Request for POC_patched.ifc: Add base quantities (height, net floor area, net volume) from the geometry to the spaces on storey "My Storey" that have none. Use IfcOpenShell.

First a look at what the model holds.

```python
import ifcopenshell
import ifcopenshell.util.element
import ifcopenshell.util.unit

model = ifcopenshell.open("POC_patched.ifc")
print(model.schema)
for unit_type in ("LENGTHUNIT", "AREAUNIT", "VOLUMEUNIT"):
    print(unit_type, ifcopenshell.util.unit.calculate_unit_scale(model, unit_type))
storey = next(s for s in model.by_type("IfcBuildingStorey") if s.Name == "My Storey")
spaces = [e for e in ifcopenshell.util.element.get_decomposition(storey) if e.is_a("IfcSpace")]
for e in sorted(spaces, key=lambda e: e.id()):
    print(e.id(), e.is_a(), e.Name, list(ifcopenshell.util.element.get_psets(e, qtos_only=True)), sep=" | ")
```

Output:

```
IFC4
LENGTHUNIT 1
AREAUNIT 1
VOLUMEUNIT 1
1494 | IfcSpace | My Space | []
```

```python
import ifcopenshell
import ifcopenshell.api.pset
import ifcopenshell.geom
import ifcopenshell.util.element
import ifcopenshell.util.shape
import ifcopenshell.util.unit

model = ifcopenshell.open("POC_patched.ifc")
unit_scale = ifcopenshell.util.unit.calculate_unit_scale(model)
area_scale = ifcopenshell.util.unit.calculate_unit_scale(model, "AREAUNIT")
volume_scale = ifcopenshell.util.unit.calculate_unit_scale(model, "VOLUMEUNIT")
settings = ifcopenshell.geom.settings()

storey = next(s for s in model.by_type("IfcBuildingStorey") if s.Name == "My Storey")
spaces = [e for e in ifcopenshell.util.element.get_decomposition(storey) if e.is_a("IfcSpace")]

for e in sorted(spaces, key=lambda e: e.id()):
    if ifcopenshell.util.element.get_psets(e, qtos_only=True, should_inherit=False):
        continue
    # Geometry comes back in metres, in the element's own axes.
    shape = ifcopenshell.geom.create_shape(settings, e)
    values = {
        "Height": ifcopenshell.util.shape.get_z(shape.geometry) / unit_scale,
        "NetFloorArea": ifcopenshell.util.shape.get_footprint_area(shape.geometry) / area_scale,
        "NetVolume": ifcopenshell.util.shape.get_volume(shape.geometry) / volume_scale,
    }
    qto = ifcopenshell.api.pset.add_qto(model, product=e, name="Qto_SpaceBaseQuantities")
    ifcopenshell.api.pset.edit_qto(model, qto=qto, properties=values)
    print(e.id(), {k: round(v, 3) for k, v in values.items()})

model.write("POC_patched_v2.ifc")
```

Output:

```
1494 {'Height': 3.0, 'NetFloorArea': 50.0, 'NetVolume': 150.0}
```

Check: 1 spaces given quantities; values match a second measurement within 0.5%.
